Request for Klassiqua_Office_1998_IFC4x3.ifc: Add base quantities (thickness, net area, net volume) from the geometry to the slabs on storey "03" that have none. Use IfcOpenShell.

First a look at what the model holds.

```python
import ifcopenshell
import ifcopenshell.util.element
import ifcopenshell.util.unit

model = ifcopenshell.open("Klassiqua_Office_1998_IFC4x3.ifc")
print(model.schema)
for unit_type in ("LENGTHUNIT", "AREAUNIT", "VOLUMEUNIT"):
    print(unit_type, ifcopenshell.util.unit.calculate_unit_scale(model, unit_type))
storey = next(s for s in model.by_type("IfcBuildingStorey") if s.Name == "03")
slabs = [e for e in ifcopenshell.util.element.get_decomposition(storey) if e.is_a("IfcSlab")]
for e in sorted(slabs, key=lambda e: e.id()):
    print(e.id(), e.is_a(), e.Name, list(ifcopenshell.util.element.get_psets(e, qtos_only=True)), sep=" | ")
```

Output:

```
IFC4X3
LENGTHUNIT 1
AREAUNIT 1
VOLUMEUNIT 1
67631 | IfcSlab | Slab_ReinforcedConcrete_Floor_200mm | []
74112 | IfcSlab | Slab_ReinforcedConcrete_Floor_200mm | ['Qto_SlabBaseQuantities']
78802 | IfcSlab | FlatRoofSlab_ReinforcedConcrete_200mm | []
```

```python
import ifcopenshell
import ifcopenshell.api.pset
import ifcopenshell.geom
import ifcopenshell.util.element
import ifcopenshell.util.shape
import ifcopenshell.util.unit

model = ifcopenshell.open("Klassiqua_Office_1998_IFC4x3.ifc")
unit_scale = ifcopenshell.util.unit.calculate_unit_scale(model)
area_scale = ifcopenshell.util.unit.calculate_unit_scale(model, "AREAUNIT")
volume_scale = ifcopenshell.util.unit.calculate_unit_scale(model, "VOLUMEUNIT")
settings = ifcopenshell.geom.settings()

storey = next(s for s in model.by_type("IfcBuildingStorey") if s.Name == "03")
slabs = [e for e in ifcopenshell.util.element.get_decomposition(storey) if e.is_a("IfcSlab")]

for e in sorted(slabs, key=lambda e: e.id()):
    if ifcopenshell.util.element.get_psets(e, qtos_only=True, should_inherit=False):
        continue
    # Geometry comes back in metres, in the element's own axes.
    shape = ifcopenshell.geom.create_shape(settings, e)
    values = {
        "Width": ifcopenshell.util.shape.get_z(shape.geometry) / unit_scale,
        "NetArea": ifcopenshell.util.shape.get_footprint_area(shape.geometry) / area_scale,
        "NetVolume": ifcopenshell.util.shape.get_volume(shape.geometry) / volume_scale,
    }
    qto = ifcopenshell.api.pset.add_qto(model, product=e, name="Qto_SlabBaseQuantities")
    ifcopenshell.api.pset.edit_qto(model, qto=qto, properties=values)
    print(e.id(), {k: round(v, 3) for k, v in values.items()})

model.write("Klassiqua_Office_1998_IFC4x3_updated.ifc")
```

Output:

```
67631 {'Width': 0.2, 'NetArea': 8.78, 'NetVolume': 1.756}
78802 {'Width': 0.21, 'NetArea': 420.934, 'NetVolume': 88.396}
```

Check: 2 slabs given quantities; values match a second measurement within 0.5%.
